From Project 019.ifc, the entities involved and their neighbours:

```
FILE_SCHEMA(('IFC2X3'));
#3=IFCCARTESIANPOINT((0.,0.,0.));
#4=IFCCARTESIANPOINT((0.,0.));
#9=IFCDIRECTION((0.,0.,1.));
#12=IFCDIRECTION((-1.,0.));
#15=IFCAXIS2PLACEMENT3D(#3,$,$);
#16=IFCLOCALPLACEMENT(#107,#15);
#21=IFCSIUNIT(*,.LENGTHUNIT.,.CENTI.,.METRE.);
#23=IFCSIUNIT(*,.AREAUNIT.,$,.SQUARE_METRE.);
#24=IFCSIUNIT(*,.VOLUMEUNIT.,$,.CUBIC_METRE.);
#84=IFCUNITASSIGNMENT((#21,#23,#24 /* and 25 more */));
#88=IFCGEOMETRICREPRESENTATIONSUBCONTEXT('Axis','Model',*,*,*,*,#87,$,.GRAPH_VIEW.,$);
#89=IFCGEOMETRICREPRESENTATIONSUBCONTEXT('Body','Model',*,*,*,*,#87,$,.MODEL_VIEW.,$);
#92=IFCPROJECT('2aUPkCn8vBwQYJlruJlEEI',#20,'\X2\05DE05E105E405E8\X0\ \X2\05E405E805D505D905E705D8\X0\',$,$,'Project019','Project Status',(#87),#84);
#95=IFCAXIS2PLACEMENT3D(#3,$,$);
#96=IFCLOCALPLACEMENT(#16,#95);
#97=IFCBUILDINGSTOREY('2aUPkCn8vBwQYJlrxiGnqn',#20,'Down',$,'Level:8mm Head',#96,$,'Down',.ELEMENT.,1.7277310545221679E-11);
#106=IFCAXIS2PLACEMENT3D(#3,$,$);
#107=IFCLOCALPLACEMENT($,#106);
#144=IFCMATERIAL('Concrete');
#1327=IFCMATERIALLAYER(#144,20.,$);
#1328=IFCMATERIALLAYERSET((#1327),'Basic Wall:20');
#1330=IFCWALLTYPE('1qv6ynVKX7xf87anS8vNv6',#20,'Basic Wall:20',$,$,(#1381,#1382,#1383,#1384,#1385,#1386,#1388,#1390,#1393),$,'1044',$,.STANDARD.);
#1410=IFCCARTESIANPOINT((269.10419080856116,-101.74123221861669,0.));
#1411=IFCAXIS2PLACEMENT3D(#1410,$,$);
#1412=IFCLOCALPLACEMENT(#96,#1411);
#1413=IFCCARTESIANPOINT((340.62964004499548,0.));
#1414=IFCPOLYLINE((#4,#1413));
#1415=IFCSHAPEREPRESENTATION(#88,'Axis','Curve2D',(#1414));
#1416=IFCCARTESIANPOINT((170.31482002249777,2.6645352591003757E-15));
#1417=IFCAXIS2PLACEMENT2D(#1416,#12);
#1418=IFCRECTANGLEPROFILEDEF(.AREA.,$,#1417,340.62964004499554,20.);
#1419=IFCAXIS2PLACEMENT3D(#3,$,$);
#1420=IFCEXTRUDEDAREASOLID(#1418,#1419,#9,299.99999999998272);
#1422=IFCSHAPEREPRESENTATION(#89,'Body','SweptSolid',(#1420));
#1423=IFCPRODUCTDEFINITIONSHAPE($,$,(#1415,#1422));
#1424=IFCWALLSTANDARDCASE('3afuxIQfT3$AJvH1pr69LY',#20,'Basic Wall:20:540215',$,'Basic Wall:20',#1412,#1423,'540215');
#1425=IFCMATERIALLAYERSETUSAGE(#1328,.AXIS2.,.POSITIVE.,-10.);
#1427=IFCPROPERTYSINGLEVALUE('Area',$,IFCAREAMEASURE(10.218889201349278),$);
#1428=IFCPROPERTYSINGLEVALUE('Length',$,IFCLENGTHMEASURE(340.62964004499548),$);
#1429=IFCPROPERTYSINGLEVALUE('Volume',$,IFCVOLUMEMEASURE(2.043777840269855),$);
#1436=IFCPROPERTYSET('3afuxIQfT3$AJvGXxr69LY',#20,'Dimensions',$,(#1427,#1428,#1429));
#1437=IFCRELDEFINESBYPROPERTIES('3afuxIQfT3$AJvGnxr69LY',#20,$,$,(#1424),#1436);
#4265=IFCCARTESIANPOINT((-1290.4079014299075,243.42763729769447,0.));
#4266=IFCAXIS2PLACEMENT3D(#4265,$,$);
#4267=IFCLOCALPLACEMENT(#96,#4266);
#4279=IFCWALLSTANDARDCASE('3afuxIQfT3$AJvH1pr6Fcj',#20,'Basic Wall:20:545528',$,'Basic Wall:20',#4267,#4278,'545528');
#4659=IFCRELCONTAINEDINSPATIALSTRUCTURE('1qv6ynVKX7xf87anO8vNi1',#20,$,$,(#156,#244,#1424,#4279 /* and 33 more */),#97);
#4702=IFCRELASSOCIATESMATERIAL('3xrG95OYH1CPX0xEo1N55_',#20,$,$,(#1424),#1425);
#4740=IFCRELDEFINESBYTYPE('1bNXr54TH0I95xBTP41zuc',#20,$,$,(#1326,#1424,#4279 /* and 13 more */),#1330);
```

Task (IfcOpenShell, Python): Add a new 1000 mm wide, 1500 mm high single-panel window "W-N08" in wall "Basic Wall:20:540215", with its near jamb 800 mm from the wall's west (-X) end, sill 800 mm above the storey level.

```python
import numpy as np
import ifcopenshell
import ifcopenshell.api.feature
import ifcopenshell.api.geometry
import ifcopenshell.api.pset
import ifcopenshell.api.root
import ifcopenshell.api.spatial
import ifcopenshell.api.type
import ifcopenshell.geom
import ifcopenshell.util.element
import ifcopenshell.util.placement
import ifcopenshell.util.representation
import ifcopenshell.util.shape
import ifcopenshell.util.unit

model = ifcopenshell.open("Project 019.ifc")
unit_scale = ifcopenshell.util.unit.calculate_unit_scale(model)
area_scale = ifcopenshell.util.unit.calculate_unit_scale(model, "AREAUNIT")
volume_scale = ifcopenshell.util.unit.calculate_unit_scale(model, "VOLUMEUNIT")
settings = ifcopenshell.geom.settings()


def volume(element):
    """Net volume in cubic metres, openings subtracted."""
    shape = ifcopenshell.geom.create_shape(settings, element)
    return ifcopenshell.util.shape.get_volume(shape.geometry)


wall = model.by_guid("3afuxIQfT3$AJvH1pr69LY")
storey = ifcopenshell.util.element.get_container(wall, ifc_class="IfcBuildingStorey")
context = ifcopenshell.util.representation.get_context(model, "Model", "Body", "MODEL_VIEW")
before = volume(wall)

width, height, from_end, sill = 1, 1.5, 0.8, 0.8  # metres

# The wall runs along its own X axis, and the end named is its -X end.
wall_shape = ifcopenshell.geom.create_shape(settings, wall)
x, y, z = ifcopenshell.util.shape.get_vertices(wall_shape.geometry).T
start = x.min() + from_end
face, thickness = float(y.min()), float(y.max() - y.min())
wall_matrix = ifcopenshell.util.placement.get_local_placement(wall.ObjectPlacement)
level = ifcopenshell.util.placement.get_local_placement(storey.ObjectPlacement)[2, 3]


def in_wall(x, y):
    """Placement at x, y metres in the wall's axes, at sill height."""
    matrix = wall_matrix.copy()
    matrix[:, 3] = wall_matrix @ np.array([x / unit_scale, y / unit_scale, 0.0, 1.0])
    matrix[2, 3] = level + sill / unit_scale
    return matrix


# Opening: a box that overshoots both wall faces by 50 mm.
opening = ifcopenshell.api.root.create_entity(model, ifc_class="IfcOpeningElement")
box = ifcopenshell.api.geometry.add_wall_representation(
    model, context=context, length=width, height=height, thickness=thickness + 0.1
)
ifcopenshell.api.geometry.assign_representation(model, product=opening, representation=box)
ifcopenshell.api.geometry.edit_object_placement(model, product=opening, matrix=in_wall(start, face - 0.05), is_si=False)
ifcopenshell.api.feature.add_feature(model, feature=opening, element=wall)

window = ifcopenshell.api.root.create_entity(model, ifc_class="IfcWindow", name="W-N08")
window.OverallWidth, window.OverallHeight = width / unit_scale, height / unit_scale
body = ifcopenshell.api.geometry.add_window_representation(
    model,
    context=context,
    overall_width=window.OverallWidth,
    overall_height=window.OverallHeight,
    partition_type="SINGLE_PANEL",
)
ifcopenshell.api.geometry.assign_representation(model, product=window, representation=body)
ifcopenshell.api.spatial.assign_container(model, products=[window], relating_structure=storey)
fills = ifcopenshell.api.feature.add_filling(model, opening=opening, element=window)
fills.OwnerHistory = window.OwnerHistory  # required in IFC2X3

# IFC2X3 keeps the operation on the window style.
style = ifcopenshell.api.root.create_entity(model, ifc_class="IfcWindowStyle", name="W-N08")
style.OperationType, style.ConstructionType = "SINGLE_PANEL", "NOTDEFINED"
style.ParameterTakesPrecedence = style.Sizeable = False
ifcopenshell.api.type.assign_type(model, related_objects=[window], relating_type=style)

# Centre the window in the wall's thickness.
ifcopenshell.api.geometry.edit_object_placement(model, product=window, matrix=in_wall(start, face), is_si=False)
window_shape = ifcopenshell.geom.create_shape(settings, window)
depth = ifcopenshell.util.shape.get_vertices(window_shape.geometry)[:, 1]
offset = face + thickness / 2 - (depth.min() + depth.max()) / 2
ifcopenshell.api.geometry.edit_object_placement(model, product=window, matrix=in_wall(start, offset), is_si=False)

after = volume(wall)

# Update the wall's stored quantities.
pset = model.by_id(ifcopenshell.util.element.get_pset(wall, "Dimensions", should_inherit=False)["id"])
ifcopenshell.api.pset.edit_pset(model, pset=pset, properties={
    "Area": model.create_entity("IfcAreaMeasure", after / thickness / area_scale),
    "Volume": model.create_entity("IfcVolumeMeasure", after / volume_scale),
})

print(f"wall volume {before:.3f} -> {after:.3f} m3")

model.write("Project 019_v2.ifc")
```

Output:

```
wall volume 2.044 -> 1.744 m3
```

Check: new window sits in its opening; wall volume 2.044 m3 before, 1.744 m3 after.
